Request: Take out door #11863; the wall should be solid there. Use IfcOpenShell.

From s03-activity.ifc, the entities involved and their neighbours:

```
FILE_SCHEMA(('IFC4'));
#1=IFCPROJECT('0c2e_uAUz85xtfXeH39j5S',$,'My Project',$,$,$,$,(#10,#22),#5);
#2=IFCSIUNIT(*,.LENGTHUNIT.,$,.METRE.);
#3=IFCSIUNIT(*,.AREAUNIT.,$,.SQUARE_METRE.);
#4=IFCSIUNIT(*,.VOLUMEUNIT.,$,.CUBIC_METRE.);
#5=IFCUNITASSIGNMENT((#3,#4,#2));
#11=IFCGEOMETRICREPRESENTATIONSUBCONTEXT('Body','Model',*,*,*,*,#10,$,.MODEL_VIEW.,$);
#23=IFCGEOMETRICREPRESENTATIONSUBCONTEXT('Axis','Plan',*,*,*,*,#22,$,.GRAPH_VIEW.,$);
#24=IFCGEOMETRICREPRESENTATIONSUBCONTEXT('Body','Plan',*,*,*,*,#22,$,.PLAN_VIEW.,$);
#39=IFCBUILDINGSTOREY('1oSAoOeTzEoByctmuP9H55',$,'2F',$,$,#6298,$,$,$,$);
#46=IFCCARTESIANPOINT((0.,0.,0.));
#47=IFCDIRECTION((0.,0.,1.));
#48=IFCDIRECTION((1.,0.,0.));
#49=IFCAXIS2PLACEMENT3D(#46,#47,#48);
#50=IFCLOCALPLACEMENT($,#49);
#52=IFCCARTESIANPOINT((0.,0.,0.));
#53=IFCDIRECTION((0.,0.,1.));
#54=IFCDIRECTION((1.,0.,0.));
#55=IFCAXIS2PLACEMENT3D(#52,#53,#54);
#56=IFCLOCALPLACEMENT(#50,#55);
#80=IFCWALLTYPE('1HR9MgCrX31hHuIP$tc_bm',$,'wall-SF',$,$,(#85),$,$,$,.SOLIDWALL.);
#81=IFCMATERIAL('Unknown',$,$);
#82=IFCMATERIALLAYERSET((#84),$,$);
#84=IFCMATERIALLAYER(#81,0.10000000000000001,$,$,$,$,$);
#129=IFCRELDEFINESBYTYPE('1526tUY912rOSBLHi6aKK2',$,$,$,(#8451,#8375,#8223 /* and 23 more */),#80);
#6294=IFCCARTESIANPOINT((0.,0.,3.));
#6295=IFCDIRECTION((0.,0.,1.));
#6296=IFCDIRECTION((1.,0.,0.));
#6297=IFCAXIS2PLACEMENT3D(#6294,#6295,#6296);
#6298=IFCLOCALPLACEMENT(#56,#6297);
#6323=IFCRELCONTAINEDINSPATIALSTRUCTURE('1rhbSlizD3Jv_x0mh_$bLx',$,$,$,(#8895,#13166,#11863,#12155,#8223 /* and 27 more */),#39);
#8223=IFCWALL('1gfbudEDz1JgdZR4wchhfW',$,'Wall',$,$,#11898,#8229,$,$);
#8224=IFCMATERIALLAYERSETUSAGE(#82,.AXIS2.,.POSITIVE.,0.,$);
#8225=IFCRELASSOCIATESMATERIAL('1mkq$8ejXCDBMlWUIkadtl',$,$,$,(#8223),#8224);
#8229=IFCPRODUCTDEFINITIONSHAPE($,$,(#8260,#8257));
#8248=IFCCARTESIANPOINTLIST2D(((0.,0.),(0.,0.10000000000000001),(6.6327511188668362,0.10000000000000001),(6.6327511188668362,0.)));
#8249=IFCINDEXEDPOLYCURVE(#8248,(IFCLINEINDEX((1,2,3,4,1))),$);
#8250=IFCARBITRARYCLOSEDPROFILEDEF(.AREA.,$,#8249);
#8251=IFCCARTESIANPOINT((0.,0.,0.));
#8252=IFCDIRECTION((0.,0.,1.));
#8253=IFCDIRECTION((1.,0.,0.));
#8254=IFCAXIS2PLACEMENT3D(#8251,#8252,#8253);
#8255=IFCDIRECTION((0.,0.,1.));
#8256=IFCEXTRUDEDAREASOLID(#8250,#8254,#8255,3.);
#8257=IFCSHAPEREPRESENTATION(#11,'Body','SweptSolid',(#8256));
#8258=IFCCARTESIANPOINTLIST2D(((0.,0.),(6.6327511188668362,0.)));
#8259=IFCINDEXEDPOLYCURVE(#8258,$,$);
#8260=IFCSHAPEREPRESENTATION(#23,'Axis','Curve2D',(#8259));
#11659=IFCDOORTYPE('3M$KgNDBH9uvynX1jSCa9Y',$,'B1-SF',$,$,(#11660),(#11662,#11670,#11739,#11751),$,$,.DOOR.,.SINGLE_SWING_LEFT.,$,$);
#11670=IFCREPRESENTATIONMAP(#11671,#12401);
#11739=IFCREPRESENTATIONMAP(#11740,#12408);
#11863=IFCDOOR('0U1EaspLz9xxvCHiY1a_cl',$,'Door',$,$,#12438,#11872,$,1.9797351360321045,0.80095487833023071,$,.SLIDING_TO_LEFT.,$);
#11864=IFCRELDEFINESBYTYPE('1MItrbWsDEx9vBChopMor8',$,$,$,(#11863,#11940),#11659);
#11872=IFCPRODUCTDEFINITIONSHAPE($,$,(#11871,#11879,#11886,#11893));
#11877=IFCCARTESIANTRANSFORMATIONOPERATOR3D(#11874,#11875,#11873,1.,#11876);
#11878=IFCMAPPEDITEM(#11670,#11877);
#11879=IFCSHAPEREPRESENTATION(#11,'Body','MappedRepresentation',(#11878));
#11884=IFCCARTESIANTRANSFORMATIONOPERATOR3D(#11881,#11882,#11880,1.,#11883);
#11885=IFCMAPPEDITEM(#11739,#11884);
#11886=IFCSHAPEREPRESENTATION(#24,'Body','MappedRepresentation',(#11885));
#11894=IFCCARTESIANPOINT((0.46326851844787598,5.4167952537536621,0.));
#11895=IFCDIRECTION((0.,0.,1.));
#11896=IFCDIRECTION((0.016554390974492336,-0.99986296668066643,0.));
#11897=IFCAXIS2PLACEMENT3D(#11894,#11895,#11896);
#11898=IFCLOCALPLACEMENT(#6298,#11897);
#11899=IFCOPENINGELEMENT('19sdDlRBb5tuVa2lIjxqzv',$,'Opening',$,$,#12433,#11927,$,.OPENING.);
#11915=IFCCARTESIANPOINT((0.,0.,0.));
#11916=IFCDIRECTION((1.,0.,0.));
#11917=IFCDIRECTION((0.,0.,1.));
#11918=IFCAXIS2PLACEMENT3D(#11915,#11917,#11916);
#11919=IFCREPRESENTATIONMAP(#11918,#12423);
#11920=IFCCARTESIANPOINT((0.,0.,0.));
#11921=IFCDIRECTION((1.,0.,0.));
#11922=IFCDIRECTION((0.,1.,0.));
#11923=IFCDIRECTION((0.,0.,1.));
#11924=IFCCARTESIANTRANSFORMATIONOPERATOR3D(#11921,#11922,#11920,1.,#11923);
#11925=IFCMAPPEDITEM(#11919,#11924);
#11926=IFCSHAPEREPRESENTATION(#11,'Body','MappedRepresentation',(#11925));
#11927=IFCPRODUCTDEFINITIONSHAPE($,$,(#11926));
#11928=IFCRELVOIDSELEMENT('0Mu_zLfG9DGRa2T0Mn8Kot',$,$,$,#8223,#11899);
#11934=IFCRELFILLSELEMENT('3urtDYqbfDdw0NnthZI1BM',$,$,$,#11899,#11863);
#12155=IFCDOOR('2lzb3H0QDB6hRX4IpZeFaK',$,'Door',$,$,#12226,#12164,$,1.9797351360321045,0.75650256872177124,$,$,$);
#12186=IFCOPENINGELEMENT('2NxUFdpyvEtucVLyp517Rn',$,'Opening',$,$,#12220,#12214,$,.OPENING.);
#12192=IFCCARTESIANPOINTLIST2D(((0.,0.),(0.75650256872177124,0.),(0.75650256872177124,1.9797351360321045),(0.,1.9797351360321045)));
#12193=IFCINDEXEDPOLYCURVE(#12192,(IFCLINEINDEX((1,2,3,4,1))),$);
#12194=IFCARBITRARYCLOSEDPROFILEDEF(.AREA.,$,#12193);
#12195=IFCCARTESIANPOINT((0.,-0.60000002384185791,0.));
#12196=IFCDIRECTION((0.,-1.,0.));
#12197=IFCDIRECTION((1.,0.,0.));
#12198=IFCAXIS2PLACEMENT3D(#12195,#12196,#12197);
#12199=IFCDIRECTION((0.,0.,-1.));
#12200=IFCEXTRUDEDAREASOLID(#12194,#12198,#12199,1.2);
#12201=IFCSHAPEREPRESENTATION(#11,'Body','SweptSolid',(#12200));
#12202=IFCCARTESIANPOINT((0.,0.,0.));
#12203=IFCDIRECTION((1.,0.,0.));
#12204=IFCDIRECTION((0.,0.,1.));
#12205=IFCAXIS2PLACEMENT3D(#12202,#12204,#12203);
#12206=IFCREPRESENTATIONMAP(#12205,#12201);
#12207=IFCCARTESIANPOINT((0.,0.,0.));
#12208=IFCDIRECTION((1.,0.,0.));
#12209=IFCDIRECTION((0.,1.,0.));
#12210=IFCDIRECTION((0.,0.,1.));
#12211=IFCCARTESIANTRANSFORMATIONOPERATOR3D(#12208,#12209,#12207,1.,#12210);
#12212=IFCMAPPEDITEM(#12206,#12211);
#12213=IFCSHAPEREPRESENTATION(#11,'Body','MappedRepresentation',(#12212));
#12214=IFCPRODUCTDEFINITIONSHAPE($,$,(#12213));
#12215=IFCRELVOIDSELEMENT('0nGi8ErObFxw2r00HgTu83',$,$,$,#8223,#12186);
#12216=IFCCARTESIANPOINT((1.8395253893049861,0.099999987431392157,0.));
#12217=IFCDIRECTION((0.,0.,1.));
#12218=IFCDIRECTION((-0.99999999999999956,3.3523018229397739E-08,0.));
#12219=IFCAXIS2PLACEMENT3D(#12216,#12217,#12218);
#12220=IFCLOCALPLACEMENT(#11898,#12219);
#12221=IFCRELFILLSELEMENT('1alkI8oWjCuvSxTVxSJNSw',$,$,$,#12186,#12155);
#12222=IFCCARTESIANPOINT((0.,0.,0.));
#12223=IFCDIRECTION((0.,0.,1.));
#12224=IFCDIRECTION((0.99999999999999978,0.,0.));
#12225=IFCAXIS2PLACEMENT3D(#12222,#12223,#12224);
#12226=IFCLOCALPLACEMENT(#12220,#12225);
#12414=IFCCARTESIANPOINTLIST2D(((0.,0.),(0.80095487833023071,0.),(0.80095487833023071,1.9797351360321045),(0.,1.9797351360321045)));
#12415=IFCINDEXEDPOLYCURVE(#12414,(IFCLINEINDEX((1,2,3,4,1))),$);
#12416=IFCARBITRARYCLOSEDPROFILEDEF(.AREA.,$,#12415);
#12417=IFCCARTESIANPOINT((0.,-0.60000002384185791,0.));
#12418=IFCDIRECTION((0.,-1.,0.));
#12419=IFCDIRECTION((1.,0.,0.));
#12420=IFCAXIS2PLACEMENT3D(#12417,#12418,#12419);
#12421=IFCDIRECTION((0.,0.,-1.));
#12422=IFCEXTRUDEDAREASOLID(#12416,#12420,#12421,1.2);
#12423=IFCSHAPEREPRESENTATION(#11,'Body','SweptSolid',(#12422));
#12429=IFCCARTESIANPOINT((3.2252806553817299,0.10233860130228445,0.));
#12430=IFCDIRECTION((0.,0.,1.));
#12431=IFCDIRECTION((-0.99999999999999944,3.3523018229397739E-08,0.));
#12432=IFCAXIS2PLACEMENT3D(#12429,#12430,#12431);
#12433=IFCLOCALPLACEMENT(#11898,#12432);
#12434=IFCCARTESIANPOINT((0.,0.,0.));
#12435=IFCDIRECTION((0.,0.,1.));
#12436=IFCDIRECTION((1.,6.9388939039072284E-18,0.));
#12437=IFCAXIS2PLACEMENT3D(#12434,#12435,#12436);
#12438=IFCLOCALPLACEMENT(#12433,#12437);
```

```python
import ifcopenshell
import ifcopenshell.api.feature
import ifcopenshell.api.root
import ifcopenshell.geom
import ifcopenshell.util.shape

model = ifcopenshell.open("s03-activity.ifc")
settings = ifcopenshell.geom.settings()


def volume(element):
    """Net volume in cubic metres, openings subtracted."""
    shape = ifcopenshell.geom.create_shape(settings, element)
    return ifcopenshell.util.shape.get_volume(shape.geometry)


door = model.by_guid("0U1EaspLz9xxvCHiY1a_cl")
opening = door.FillsVoids[0].RelatingOpeningElement
wall = opening.VoidsElements[0].RelatingBuildingElement
before = volume(wall)

ifcopenshell.api.root.remove_product(model, product=door)
ifcopenshell.api.feature.remove_feature(model, feature=opening)

after = volume(wall)

print(f"wall volume {before:.3f} -> {after:.3f} m3")

model.write("s03-activity_rev.ifc")
```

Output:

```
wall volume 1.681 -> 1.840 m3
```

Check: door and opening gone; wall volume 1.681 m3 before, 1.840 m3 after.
